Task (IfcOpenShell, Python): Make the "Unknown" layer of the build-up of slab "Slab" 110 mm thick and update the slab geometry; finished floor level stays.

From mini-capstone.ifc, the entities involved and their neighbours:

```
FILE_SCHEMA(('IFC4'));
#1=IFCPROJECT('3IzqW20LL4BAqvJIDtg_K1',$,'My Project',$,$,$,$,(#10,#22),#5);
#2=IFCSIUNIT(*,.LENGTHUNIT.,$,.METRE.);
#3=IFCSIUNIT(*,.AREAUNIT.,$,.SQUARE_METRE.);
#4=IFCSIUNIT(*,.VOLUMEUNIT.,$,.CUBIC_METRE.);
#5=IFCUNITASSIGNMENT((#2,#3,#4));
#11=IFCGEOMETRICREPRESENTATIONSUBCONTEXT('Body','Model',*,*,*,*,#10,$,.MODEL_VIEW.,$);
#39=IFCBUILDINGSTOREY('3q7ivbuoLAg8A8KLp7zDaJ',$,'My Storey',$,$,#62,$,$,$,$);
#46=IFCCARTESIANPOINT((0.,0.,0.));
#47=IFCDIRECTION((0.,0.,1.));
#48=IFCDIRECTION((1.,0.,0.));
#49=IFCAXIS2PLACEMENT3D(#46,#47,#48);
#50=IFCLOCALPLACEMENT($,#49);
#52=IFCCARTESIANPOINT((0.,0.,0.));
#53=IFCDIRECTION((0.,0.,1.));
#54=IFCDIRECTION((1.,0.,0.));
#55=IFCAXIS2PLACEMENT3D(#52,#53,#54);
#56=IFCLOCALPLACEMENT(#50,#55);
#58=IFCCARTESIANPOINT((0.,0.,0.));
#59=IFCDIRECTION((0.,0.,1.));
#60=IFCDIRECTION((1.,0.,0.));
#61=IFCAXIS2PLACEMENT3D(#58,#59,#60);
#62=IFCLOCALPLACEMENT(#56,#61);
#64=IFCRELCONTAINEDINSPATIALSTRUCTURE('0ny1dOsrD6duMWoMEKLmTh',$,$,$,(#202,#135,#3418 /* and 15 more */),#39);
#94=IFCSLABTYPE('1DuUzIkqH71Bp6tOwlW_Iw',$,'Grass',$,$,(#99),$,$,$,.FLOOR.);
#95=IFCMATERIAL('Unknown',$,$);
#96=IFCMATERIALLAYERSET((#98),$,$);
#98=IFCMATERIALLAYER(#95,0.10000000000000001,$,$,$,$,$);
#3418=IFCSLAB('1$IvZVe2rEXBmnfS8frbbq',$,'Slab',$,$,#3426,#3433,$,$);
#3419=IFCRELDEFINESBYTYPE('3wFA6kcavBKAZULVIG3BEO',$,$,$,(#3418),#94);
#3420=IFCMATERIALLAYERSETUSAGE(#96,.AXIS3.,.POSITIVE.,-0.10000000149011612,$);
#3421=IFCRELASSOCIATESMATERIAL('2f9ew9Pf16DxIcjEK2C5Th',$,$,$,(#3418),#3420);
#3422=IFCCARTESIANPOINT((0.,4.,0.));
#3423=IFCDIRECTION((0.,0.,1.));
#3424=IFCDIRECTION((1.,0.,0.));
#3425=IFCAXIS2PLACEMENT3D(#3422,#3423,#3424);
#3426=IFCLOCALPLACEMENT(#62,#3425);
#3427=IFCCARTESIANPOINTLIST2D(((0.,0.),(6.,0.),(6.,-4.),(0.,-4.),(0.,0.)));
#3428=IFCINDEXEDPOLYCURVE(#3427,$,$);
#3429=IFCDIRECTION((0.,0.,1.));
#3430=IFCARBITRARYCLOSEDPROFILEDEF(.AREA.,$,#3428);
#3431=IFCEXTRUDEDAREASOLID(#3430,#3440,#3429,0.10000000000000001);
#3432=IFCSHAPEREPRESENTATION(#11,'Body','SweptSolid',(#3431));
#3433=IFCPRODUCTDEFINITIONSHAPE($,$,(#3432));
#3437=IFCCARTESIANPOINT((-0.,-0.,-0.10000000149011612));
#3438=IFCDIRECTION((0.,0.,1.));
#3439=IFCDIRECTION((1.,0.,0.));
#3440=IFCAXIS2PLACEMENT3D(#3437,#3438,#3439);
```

```python
import ifcopenshell
import ifcopenshell.util.element
import ifcopenshell.util.representation
import ifcopenshell.util.unit

model = ifcopenshell.open("mini-capstone.ifc")
unit_scale = ifcopenshell.util.unit.calculate_unit_scale(model)

layer_set = model.by_id(96)
layer = next(l for l in layer_set.MaterialLayers if l.Material and l.Material.Name == "Unknown")
change = 0.11 / unit_scale - layer.LayerThickness
layer.LayerThickness += change

# Geometry does not follow the layer set by itself.
slabs = [e for e in ifcopenshell.util.element.get_elements_by_material(model, layer_set) if e.is_a("IfcSlab")]
for slab in sorted(slabs, key=lambda e: e.id()):
    body = ifcopenshell.util.representation.get_representation(slab, "Model", "Body")
    solid = body.Items[0]
    old_depth = solid.Depth
    solid.Depth += change
    # Extruded upwards: lower the start of the extrusion so the top stays.
    x, y, z = solid.Position.Location.Coordinates
    solid.Position.Location = model.createIfcCartesianPoint((x, y, z - change))
    print(slab.id(), f"{old_depth:g} -> {solid.Depth:g}")

# The layers are counted up from the underside, which has moved.
for usage in {ifcopenshell.util.element.get_material(slab) for slab in slabs}:
    usage.OffsetFromReferenceLine -= change

model.write("mini-capstone-out.ifc")
```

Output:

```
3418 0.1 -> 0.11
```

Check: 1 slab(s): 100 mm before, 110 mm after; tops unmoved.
